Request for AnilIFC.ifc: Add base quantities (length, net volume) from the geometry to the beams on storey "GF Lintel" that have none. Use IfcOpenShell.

First a look at what the model holds.

```python
import ifcopenshell
import ifcopenshell.util.element
import ifcopenshell.util.unit

model = ifcopenshell.open("AnilIFC.ifc")
print(model.schema)
for unit_type in ("LENGTHUNIT", "AREAUNIT", "VOLUMEUNIT"):
    print(unit_type, ifcopenshell.util.unit.calculate_unit_scale(model, unit_type))
storey = next(s for s in model.by_type("IfcBuildingStorey") if s.Name == "GF Lintel")
beams = [e for e in ifcopenshell.util.element.get_decomposition(storey) if e.is_a("IfcBeam")]
for e in sorted(beams, key=lambda e: e.id()):
    print(e.id(), e.is_a(), e.Name, list(ifcopenshell.util.element.get_psets(e, qtos_only=True)), sep=" | ")
```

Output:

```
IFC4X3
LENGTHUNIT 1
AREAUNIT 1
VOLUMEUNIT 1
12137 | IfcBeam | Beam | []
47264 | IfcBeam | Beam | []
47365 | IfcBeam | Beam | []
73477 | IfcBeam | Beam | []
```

```python
import ifcopenshell
import ifcopenshell.api.pset
import ifcopenshell.geom
import ifcopenshell.util.element
import ifcopenshell.util.shape
import ifcopenshell.util.unit

model = ifcopenshell.open("AnilIFC.ifc")
unit_scale = ifcopenshell.util.unit.calculate_unit_scale(model)
volume_scale = ifcopenshell.util.unit.calculate_unit_scale(model, "VOLUMEUNIT")
settings = ifcopenshell.geom.settings()

storey = next(s for s in model.by_type("IfcBuildingStorey") if s.Name == "GF Lintel")
beams = [e for e in ifcopenshell.util.element.get_decomposition(storey) if e.is_a("IfcBeam")]

for e in sorted(beams, key=lambda e: e.id()):
    if ifcopenshell.util.element.get_psets(e, qtos_only=True, should_inherit=False):
        continue
    # Geometry comes back in metres, in the element's own axes.
    shape = ifcopenshell.geom.create_shape(settings, e)
    values = {
        "Length": ifcopenshell.util.shape.get_max_xyz(shape.geometry) / unit_scale,
        "NetVolume": ifcopenshell.util.shape.get_volume(shape.geometry) / volume_scale,
    }
    qto = ifcopenshell.api.pset.add_qto(model, product=e, name="Qto_BeamBaseQuantities")
    ifcopenshell.api.pset.edit_qto(model, qto=qto, properties=values)
    print(e.id(), {k: round(v, 3) for k, v in values.items()})

model.write("AnilIFC_v2.ifc")
```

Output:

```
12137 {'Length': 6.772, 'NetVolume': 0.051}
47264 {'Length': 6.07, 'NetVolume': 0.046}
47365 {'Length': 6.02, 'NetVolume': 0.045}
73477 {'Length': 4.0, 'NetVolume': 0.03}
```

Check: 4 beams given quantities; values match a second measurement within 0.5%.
